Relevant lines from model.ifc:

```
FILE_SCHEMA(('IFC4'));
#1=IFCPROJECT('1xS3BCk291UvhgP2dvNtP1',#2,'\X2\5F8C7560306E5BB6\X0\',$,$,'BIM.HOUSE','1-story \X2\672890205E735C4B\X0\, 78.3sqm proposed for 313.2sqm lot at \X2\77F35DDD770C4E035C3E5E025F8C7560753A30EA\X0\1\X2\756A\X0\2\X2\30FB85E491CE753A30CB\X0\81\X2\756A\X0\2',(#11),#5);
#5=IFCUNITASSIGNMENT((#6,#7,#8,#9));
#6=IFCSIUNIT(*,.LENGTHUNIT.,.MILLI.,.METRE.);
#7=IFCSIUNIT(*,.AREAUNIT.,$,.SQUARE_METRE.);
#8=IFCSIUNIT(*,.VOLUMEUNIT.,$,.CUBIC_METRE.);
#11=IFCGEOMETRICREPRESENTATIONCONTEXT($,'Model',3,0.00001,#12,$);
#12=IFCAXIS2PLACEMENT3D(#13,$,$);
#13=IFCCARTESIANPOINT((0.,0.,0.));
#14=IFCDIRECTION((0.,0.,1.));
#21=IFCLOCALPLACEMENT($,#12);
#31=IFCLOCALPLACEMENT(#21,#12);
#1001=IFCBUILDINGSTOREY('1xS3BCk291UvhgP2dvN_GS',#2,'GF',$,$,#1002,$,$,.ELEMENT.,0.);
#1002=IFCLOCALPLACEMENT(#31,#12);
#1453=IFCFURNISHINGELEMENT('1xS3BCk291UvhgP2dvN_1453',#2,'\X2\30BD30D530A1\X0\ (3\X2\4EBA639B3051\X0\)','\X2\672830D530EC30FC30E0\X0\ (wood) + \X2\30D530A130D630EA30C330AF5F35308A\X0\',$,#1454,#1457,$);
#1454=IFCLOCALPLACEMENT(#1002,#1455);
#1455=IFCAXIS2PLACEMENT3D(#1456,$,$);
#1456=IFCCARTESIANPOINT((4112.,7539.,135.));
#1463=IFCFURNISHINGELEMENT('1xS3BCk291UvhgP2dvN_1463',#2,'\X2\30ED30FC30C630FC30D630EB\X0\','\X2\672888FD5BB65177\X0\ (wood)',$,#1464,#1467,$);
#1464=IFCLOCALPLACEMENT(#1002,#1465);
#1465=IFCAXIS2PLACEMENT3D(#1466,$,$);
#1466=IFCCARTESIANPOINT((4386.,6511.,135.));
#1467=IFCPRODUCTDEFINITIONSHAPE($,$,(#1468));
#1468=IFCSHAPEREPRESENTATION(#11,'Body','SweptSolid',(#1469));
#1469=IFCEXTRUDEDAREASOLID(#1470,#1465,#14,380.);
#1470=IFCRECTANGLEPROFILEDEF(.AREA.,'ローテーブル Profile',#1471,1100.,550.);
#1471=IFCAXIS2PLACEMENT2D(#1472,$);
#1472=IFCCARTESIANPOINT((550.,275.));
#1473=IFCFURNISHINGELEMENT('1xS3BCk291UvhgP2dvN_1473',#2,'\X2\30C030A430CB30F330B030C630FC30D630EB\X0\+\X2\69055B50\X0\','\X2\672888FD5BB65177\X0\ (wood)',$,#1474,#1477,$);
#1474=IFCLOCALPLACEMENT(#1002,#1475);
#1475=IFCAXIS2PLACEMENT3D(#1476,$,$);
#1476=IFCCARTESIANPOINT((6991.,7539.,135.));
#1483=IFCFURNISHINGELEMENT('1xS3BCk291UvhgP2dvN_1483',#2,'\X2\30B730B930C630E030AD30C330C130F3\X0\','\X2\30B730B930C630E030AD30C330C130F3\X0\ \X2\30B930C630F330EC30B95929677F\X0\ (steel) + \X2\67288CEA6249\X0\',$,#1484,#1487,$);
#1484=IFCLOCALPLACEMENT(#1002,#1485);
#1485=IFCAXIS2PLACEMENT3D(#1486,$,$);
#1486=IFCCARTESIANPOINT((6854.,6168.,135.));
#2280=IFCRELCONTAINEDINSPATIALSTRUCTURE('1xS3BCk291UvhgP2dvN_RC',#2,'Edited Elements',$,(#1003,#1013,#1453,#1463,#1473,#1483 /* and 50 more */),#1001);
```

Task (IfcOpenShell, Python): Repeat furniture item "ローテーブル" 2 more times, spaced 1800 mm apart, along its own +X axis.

```python
import ifcopenshell
import ifcopenshell.api.geometry
import ifcopenshell.api.root
import ifcopenshell.util.element
import ifcopenshell.util.placement
import ifcopenshell.util.unit

model = ifcopenshell.open("model.ifc")
unit_scale = ifcopenshell.util.unit.calculate_unit_scale(model)


def reuse_history(source, copy):
    """copy_class also copies each property set's owner history, people and application; keep the originals."""
    for rel in copy.IsDefinedBy:
        if rel.is_a("IfcRelDefinesByProperties") and (history := rel.RelatingPropertyDefinition.OwnerHistory):
            rel.RelatingPropertyDefinition.OwnerHistory = source.OwnerHistory
            ifcopenshell.util.element.remove_deep2(model, history)


source = model.by_guid("1xS3BCk291UvhgP2dvN_1463")
base = ifcopenshell.util.placement.get_local_placement(source.ObjectPlacement)
step = base[:3, 0] * 1.8 / unit_scale

for i in range(1, 3):
    copy = ifcopenshell.api.root.copy_class(model, product=source)
    copy.Representation = ifcopenshell.util.element.copy_deep(
        model, source.Representation, exclude=["IfcGeometricRepresentationContext", "IfcRepresentationMap"]
    )
    reuse_history(source, copy)
    matrix = base.copy()
    matrix[:3, 3] += i * step
    print("added at", matrix[:3, 3].round(3) + 0.0)
    ifcopenshell.api.geometry.edit_object_placement(model, product=copy, matrix=matrix, is_si=False)

model.write("model_edited.ifc")
```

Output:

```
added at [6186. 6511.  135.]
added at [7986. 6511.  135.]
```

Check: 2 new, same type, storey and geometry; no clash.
